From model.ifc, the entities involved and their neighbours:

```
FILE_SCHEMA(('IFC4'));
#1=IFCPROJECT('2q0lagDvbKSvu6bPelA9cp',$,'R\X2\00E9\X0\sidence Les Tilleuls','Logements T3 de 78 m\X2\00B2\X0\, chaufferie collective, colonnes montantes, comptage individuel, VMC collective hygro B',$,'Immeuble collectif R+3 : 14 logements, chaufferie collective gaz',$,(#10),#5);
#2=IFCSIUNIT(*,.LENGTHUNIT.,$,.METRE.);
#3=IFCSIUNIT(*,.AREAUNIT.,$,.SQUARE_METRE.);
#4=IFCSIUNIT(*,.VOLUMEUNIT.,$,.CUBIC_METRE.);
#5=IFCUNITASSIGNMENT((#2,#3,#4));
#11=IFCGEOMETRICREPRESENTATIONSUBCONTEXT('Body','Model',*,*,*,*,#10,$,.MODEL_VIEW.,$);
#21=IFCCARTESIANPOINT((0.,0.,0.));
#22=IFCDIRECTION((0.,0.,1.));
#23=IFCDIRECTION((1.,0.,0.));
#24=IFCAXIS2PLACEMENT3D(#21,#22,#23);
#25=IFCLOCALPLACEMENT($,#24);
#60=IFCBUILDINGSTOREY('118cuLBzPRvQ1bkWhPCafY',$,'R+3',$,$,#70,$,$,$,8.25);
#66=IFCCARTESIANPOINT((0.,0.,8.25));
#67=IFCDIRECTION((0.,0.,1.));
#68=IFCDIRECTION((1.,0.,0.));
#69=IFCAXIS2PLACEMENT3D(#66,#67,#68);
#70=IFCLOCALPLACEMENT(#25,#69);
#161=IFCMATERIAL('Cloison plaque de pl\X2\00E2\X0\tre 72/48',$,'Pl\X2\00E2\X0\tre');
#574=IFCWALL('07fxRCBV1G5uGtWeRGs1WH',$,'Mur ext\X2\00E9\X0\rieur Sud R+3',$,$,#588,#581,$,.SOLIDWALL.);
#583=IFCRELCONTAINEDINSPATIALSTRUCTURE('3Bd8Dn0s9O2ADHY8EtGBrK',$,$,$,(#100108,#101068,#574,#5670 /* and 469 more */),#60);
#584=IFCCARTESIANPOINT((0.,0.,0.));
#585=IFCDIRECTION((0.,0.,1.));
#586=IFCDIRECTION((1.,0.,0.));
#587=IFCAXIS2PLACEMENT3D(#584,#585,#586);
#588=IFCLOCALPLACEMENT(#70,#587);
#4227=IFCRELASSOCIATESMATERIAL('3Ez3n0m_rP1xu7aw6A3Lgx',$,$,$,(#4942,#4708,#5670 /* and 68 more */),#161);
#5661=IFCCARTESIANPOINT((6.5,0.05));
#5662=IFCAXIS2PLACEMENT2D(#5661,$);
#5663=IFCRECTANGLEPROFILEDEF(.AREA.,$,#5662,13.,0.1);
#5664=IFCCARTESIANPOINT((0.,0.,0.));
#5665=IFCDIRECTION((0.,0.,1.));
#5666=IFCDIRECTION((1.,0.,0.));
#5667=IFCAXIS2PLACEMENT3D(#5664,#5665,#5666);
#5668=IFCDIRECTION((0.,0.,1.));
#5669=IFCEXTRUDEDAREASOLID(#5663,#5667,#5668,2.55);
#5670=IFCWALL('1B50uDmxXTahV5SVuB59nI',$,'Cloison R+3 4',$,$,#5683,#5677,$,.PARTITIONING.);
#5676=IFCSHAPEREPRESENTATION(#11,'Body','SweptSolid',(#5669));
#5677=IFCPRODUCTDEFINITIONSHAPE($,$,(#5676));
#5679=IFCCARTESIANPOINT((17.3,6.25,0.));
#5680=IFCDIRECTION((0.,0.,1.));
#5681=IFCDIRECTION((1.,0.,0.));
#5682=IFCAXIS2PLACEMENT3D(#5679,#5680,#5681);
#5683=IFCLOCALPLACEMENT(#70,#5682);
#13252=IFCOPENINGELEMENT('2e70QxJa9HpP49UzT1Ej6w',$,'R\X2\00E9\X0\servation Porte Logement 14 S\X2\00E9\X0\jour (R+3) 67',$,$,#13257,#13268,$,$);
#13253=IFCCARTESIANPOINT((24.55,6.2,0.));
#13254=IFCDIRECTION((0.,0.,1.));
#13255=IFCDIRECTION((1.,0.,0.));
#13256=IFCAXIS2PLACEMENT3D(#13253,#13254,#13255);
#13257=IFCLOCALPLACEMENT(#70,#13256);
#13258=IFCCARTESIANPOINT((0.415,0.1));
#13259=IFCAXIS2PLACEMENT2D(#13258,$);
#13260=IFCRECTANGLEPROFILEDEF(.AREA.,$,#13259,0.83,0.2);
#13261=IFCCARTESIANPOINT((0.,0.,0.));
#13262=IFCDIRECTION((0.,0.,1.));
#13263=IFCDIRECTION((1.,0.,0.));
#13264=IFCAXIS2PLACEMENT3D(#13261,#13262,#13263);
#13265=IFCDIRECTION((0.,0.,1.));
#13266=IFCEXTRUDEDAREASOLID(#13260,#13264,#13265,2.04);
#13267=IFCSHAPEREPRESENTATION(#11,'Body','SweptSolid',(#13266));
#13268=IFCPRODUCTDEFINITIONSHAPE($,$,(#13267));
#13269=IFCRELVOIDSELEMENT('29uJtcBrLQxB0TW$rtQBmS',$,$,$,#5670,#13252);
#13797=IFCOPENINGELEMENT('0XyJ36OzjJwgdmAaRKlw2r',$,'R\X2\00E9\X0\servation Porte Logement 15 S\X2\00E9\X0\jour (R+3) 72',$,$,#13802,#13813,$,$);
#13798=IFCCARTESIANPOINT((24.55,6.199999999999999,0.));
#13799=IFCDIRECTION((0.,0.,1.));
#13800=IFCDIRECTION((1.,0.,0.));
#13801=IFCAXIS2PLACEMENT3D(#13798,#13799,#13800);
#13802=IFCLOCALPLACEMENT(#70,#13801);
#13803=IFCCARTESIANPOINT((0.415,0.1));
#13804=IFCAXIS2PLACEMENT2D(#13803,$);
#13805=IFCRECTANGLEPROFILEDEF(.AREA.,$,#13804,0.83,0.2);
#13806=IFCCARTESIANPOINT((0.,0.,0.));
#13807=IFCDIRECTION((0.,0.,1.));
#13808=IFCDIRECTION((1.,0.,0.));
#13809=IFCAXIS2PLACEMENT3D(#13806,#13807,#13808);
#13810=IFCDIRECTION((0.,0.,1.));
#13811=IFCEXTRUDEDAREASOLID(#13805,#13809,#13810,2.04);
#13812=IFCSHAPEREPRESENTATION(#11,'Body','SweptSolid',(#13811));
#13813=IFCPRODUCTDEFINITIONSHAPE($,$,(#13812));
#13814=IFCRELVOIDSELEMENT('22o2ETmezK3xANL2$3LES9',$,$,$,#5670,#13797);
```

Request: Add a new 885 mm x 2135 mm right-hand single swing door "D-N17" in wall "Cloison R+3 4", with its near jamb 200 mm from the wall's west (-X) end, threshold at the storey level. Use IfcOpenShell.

```python
import numpy as np
import ifcopenshell
import ifcopenshell.api.feature
import ifcopenshell.api.geometry
import ifcopenshell.api.root
import ifcopenshell.api.spatial
import ifcopenshell.geom
import ifcopenshell.util.element
import ifcopenshell.util.placement
import ifcopenshell.util.representation
import ifcopenshell.util.shape
import ifcopenshell.util.unit

model = ifcopenshell.open("model.ifc")
unit_scale = ifcopenshell.util.unit.calculate_unit_scale(model)
settings = ifcopenshell.geom.settings()


def volume(element):
    """Net volume in cubic metres, openings subtracted."""
    shape = ifcopenshell.geom.create_shape(settings, element)
    return ifcopenshell.util.shape.get_volume(shape.geometry)


wall = model.by_guid("1B50uDmxXTahV5SVuB59nI")
storey = ifcopenshell.util.element.get_container(wall, ifc_class="IfcBuildingStorey")
context = ifcopenshell.util.representation.get_context(model, "Model", "Body", "MODEL_VIEW")
before = volume(wall)

width, height, from_end, sill = 0.885, 2.135, 0.2, 0.0  # metres

# The wall runs along its own X axis, and the end named is its -X end.
wall_shape = ifcopenshell.geom.create_shape(settings, wall)
x, y, z = ifcopenshell.util.shape.get_vertices(wall_shape.geometry).T
start = x.min() + from_end
face, thickness = float(y.min()), float(y.max() - y.min())
wall_matrix = ifcopenshell.util.placement.get_local_placement(wall.ObjectPlacement)
level = ifcopenshell.util.placement.get_local_placement(storey.ObjectPlacement)[2, 3]


def in_wall(x, y):
    """Placement at x, y metres in the wall's axes, at sill height."""
    matrix = wall_matrix.copy()
    matrix[:, 3] = wall_matrix @ np.array([x / unit_scale, y / unit_scale, 0.0, 1.0])
    matrix[2, 3] = level + sill / unit_scale
    return matrix


# Opening: a box that overshoots both wall faces by 50 mm.
opening = ifcopenshell.api.root.create_entity(model, ifc_class="IfcOpeningElement", predefined_type="OPENING")
box = ifcopenshell.api.geometry.add_wall_representation(
    model, context=context, length=width, height=height, thickness=thickness + 0.1
)
ifcopenshell.api.geometry.assign_representation(model, product=opening, representation=box)
ifcopenshell.api.geometry.edit_object_placement(model, product=opening, matrix=in_wall(start, face - 0.05), is_si=False)
ifcopenshell.api.feature.add_feature(model, feature=opening, element=wall)

door = ifcopenshell.api.root.create_entity(model, ifc_class="IfcDoor", name="D-N17", predefined_type="DOOR")
door.OverallWidth, door.OverallHeight = width / unit_scale, height / unit_scale
door.OperationType = "SINGLE_SWING_RIGHT"
body = ifcopenshell.api.geometry.add_door_representation(
    model,
    context=context,
    overall_width=door.OverallWidth,
    overall_height=door.OverallHeight,
    operation_type="SINGLE_SWING_RIGHT",
    lining_properties={"LiningDepth": thickness / unit_scale, "ThresholdDepth": thickness / unit_scale},
)
ifcopenshell.api.geometry.assign_representation(model, product=door, representation=body)
ifcopenshell.api.spatial.assign_container(model, products=[door], relating_structure=storey)
ifcopenshell.api.feature.add_filling(model, opening=opening, element=door)

# The lining spans the wall, so the door starts at the wall face.
ifcopenshell.api.geometry.edit_object_placement(model, product=door, matrix=in_wall(start, face), is_si=False)

after = volume(wall)

print(f"wall volume {before:.3f} -> {after:.3f} m3")

model.write("model-out.ifc")
```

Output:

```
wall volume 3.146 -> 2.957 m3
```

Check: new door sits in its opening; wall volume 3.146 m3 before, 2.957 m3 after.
